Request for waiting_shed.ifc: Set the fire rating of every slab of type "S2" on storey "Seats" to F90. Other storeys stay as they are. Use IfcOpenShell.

First a look at what the model holds.

```python
import ifcopenshell
import ifcopenshell.util.element

model = ifcopenshell.open("waiting_shed.ifc")
print(model.schema)
storey = next(s for s in model.by_type("IfcBuildingStorey") if s.Name == "Seats")
slabs = [e for e in ifcopenshell.util.element.get_decomposition(storey) if e.is_a("IfcSlab")]
seen = {}
for e in slabs:
    element_type = ifcopenshell.util.element.get_type(e)
    key = (element_type.Name if element_type != e and element_type else None, ifcopenshell.util.element.get_pset(e, "Pset_SlabCommon", "FireRating"))
    seen[key] = seen.get(key, 0) + 1
for (name, value), count in sorted(seen.items(), key=str):
    print(count, "x", name, "|", value)
```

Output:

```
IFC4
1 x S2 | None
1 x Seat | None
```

```python
import ifcopenshell
import ifcopenshell.api.pset
import ifcopenshell.util.element

model = ifcopenshell.open("waiting_shed.ifc")

storey = next(s for s in model.by_type("IfcBuildingStorey") if s.Name == "Seats")
slabs = [e for e in ifcopenshell.util.element.get_decomposition(storey) if e.is_a("IfcSlab")]

count = 0
for e in slabs:
    element_type = ifcopenshell.util.element.get_type(e)
    if element_type in (None, e) or element_type.Name != "S2":
        continue
    # add_pset returns the element's existing set when there is one.
    pset = ifcopenshell.api.pset.add_pset(model, product=e, name="Pset_SlabCommon")
    ifcopenshell.api.pset.edit_pset(model, pset=pset, properties={"FireRating": "F90"})
    count += 1

print(count, "slabs updated")

model.write("waiting_shed_v2.ifc")
```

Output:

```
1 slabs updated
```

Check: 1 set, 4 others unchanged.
